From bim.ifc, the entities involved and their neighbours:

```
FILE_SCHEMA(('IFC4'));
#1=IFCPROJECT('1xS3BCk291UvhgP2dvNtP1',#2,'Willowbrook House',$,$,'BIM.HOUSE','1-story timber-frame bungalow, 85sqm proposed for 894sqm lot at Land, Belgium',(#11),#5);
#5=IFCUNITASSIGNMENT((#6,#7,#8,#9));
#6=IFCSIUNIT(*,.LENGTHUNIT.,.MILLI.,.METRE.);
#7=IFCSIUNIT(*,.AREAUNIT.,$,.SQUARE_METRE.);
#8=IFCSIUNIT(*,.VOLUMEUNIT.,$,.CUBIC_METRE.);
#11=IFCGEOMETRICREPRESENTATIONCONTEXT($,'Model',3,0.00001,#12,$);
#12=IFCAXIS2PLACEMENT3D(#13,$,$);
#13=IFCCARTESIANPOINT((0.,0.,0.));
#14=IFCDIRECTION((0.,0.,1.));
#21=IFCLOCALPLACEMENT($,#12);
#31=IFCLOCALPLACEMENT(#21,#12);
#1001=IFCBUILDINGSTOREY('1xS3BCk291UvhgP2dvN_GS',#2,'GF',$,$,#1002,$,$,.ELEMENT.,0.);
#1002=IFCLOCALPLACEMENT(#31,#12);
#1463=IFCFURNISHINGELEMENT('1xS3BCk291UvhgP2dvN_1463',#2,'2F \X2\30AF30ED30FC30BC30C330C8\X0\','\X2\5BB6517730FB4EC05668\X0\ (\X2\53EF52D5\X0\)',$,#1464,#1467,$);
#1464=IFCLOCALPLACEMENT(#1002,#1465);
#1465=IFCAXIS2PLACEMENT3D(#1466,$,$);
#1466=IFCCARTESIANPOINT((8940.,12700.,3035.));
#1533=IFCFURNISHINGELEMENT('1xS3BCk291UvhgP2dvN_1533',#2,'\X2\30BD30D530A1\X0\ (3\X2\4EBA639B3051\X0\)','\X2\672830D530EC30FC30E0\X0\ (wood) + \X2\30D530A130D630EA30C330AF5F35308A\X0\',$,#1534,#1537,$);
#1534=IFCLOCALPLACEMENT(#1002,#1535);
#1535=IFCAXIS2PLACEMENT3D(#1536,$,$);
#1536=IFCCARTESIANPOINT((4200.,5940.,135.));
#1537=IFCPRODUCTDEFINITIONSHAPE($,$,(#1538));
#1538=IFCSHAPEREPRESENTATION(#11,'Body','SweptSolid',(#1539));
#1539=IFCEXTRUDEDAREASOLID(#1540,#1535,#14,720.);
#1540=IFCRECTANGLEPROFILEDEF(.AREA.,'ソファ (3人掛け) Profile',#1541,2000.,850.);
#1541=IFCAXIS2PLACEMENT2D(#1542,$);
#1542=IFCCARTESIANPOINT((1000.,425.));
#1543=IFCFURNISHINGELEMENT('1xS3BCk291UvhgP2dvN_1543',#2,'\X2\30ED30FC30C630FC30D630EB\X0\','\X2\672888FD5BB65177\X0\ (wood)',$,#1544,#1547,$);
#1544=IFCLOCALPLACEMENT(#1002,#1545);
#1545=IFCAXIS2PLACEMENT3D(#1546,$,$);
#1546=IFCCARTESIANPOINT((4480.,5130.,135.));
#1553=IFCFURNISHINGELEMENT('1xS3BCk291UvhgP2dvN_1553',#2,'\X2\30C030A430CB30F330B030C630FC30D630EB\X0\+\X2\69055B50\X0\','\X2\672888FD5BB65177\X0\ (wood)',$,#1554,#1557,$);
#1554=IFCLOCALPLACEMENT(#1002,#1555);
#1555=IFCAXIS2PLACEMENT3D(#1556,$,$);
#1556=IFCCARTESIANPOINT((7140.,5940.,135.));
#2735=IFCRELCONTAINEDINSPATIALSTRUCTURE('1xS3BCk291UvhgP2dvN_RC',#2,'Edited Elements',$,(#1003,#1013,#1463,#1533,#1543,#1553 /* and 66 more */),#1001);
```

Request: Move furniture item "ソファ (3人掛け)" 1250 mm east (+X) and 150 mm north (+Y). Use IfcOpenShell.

```python
import ifcopenshell
import ifcopenshell.api.geometry
import ifcopenshell.util.placement

model = ifcopenshell.open("bim.ifc")

item = model.by_id(1533)
matrix = ifcopenshell.util.placement.get_local_placement(item.ObjectPlacement)
matrix[0, 3] += 1250.0
matrix[1, 3] += 150.0
ifcopenshell.api.geometry.edit_object_placement(model, product=item, matrix=matrix, is_si=False)

print(ifcopenshell.util.placement.get_local_placement(item.ObjectPlacement).round(3) + 0.0)

model.write("bim-out.ifc")
```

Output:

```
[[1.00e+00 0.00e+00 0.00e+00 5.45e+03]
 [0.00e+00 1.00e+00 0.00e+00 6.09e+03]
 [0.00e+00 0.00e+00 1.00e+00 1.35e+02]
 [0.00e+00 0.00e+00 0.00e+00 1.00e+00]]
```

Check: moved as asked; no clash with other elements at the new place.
